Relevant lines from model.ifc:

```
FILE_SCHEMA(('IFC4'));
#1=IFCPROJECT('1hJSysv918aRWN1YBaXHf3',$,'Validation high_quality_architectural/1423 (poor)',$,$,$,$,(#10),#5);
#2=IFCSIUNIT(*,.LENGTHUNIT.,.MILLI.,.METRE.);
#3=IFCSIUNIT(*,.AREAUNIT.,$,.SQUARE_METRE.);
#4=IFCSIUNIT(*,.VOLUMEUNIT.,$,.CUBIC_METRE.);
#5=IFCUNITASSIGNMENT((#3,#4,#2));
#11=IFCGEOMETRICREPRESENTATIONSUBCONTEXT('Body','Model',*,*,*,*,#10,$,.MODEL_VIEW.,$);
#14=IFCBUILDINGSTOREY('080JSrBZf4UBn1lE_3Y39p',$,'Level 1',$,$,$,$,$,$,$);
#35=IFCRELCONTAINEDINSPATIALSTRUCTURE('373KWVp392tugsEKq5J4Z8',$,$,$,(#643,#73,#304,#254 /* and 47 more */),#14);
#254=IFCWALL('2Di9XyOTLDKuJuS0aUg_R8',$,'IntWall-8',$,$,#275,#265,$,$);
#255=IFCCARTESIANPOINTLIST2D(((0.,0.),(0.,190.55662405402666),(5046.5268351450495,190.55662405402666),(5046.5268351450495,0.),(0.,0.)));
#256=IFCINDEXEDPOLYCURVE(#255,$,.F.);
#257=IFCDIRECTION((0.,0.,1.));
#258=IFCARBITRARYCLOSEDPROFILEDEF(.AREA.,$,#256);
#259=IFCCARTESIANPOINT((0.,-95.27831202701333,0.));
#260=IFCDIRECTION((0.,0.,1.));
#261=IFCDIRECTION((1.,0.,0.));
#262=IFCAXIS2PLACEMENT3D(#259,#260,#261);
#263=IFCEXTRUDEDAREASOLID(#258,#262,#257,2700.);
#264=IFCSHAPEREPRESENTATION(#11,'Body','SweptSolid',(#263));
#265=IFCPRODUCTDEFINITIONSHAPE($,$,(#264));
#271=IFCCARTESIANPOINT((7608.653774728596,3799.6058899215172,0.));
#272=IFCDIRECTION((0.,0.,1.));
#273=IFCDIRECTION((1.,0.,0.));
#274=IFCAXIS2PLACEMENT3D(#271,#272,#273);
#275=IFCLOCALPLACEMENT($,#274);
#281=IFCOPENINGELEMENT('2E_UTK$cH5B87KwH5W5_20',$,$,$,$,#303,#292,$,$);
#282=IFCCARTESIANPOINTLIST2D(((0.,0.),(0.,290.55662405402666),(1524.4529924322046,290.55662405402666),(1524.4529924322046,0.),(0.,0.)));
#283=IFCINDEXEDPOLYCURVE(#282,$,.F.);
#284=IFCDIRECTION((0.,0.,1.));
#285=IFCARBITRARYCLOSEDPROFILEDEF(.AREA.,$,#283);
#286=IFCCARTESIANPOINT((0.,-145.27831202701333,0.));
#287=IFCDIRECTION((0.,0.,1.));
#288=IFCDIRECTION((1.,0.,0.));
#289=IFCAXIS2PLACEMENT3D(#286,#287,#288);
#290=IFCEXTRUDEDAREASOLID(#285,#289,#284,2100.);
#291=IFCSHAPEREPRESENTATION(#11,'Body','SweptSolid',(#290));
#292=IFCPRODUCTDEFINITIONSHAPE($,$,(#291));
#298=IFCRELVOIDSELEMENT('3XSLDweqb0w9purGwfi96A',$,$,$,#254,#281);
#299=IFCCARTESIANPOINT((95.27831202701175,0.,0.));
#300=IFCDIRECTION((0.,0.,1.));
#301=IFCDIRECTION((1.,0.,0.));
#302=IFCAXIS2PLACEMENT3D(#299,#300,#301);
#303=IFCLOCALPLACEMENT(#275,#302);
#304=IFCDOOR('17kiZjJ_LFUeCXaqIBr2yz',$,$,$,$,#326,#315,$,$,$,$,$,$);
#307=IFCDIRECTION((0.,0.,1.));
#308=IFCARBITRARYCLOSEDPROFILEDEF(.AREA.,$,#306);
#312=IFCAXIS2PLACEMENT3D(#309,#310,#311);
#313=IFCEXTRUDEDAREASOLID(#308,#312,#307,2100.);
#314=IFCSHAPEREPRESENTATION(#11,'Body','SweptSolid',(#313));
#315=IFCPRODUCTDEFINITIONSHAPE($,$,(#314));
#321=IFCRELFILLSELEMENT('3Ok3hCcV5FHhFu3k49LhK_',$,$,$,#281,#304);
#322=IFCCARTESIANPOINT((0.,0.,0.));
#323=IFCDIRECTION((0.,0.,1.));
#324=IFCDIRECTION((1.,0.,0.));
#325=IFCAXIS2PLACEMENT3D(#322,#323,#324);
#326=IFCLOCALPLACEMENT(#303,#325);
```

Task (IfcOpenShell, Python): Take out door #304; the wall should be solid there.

```python
import ifcopenshell
import ifcopenshell.api.feature
import ifcopenshell.api.root
import ifcopenshell.geom
import ifcopenshell.util.shape

model = ifcopenshell.open("model.ifc")
settings = ifcopenshell.geom.settings()


def volume(element):
    """Net volume in cubic metres, openings subtracted."""
    shape = ifcopenshell.geom.create_shape(settings, element)
    return ifcopenshell.util.shape.get_volume(shape.geometry)


door = model.by_guid("17kiZjJ_LFUeCXaqIBr2yz")
opening = door.FillsVoids[0].RelatingOpeningElement
wall = opening.VoidsElements[0].RelatingBuildingElement
before = volume(wall)

ifcopenshell.api.root.remove_product(model, product=door)
ifcopenshell.api.feature.remove_feature(model, feature=opening)

after = volume(wall)

print(f"wall volume {before:.3f} -> {after:.3f} m3")

model.write("model_v2.ifc")
```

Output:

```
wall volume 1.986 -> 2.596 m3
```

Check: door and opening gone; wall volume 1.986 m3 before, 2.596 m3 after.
